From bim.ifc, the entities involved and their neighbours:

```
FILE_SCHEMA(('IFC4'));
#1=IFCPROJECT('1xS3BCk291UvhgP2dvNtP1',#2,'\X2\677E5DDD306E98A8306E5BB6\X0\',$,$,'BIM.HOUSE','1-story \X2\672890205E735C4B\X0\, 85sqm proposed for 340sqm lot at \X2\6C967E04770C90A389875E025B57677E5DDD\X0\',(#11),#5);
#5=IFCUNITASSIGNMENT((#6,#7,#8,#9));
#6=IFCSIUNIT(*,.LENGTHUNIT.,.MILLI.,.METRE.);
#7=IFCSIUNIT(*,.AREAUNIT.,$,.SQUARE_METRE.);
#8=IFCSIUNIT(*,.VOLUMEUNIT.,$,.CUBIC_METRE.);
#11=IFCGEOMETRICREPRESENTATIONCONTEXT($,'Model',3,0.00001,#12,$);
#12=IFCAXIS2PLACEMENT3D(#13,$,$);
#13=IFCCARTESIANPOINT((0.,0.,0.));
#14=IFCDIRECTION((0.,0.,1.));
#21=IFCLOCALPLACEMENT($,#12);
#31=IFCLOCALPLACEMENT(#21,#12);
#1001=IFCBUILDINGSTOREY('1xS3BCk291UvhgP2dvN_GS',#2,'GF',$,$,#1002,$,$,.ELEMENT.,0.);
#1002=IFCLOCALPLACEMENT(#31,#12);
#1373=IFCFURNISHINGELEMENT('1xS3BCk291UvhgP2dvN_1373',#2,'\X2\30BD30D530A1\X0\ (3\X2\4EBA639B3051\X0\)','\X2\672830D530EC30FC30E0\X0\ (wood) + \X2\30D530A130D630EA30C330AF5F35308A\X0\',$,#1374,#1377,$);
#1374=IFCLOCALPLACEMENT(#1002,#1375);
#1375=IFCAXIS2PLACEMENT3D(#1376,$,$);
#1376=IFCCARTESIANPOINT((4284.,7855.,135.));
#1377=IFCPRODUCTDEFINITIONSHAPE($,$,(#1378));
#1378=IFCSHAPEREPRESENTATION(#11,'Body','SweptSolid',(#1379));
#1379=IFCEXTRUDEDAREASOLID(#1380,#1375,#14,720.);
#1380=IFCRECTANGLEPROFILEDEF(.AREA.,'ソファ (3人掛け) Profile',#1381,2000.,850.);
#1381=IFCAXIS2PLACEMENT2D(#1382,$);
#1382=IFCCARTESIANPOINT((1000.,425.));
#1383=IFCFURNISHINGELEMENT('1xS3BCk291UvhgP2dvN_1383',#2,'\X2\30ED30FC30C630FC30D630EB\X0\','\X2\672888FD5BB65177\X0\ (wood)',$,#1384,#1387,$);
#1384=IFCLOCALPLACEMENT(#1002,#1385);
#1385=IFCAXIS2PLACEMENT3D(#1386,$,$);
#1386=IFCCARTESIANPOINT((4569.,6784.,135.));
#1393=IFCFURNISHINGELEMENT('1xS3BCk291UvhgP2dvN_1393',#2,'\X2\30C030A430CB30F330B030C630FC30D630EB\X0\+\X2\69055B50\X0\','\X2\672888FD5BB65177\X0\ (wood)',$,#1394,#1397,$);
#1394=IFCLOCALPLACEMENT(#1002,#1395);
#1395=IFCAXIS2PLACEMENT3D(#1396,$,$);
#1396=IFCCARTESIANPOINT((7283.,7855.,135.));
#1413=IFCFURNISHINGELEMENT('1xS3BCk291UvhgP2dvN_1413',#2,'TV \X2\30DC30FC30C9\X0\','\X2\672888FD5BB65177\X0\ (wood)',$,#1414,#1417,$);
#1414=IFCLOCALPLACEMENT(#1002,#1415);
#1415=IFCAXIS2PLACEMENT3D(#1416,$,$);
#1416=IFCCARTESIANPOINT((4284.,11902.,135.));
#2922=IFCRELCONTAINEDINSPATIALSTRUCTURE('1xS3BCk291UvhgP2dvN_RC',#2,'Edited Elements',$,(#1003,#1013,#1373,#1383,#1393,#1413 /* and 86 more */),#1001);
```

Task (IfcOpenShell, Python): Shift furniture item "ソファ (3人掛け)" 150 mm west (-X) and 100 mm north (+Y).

```python
import ifcopenshell
import ifcopenshell.api.geometry
import ifcopenshell.util.placement

model = ifcopenshell.open("bim.ifc")

item = model.by_guid("1xS3BCk291UvhgP2dvN_1373")
matrix = ifcopenshell.util.placement.get_local_placement(item.ObjectPlacement)
matrix[0, 3] -= 150.0
matrix[1, 3] += 100.0
ifcopenshell.api.geometry.edit_object_placement(model, product=item, matrix=matrix, is_si=False)

print(ifcopenshell.util.placement.get_local_placement(item.ObjectPlacement).round(3) + 0.0)

model.write("bim_v2.ifc")
```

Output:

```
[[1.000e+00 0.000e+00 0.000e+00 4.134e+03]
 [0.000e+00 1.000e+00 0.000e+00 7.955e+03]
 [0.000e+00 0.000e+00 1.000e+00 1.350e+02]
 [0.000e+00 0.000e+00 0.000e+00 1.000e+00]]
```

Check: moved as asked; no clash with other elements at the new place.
